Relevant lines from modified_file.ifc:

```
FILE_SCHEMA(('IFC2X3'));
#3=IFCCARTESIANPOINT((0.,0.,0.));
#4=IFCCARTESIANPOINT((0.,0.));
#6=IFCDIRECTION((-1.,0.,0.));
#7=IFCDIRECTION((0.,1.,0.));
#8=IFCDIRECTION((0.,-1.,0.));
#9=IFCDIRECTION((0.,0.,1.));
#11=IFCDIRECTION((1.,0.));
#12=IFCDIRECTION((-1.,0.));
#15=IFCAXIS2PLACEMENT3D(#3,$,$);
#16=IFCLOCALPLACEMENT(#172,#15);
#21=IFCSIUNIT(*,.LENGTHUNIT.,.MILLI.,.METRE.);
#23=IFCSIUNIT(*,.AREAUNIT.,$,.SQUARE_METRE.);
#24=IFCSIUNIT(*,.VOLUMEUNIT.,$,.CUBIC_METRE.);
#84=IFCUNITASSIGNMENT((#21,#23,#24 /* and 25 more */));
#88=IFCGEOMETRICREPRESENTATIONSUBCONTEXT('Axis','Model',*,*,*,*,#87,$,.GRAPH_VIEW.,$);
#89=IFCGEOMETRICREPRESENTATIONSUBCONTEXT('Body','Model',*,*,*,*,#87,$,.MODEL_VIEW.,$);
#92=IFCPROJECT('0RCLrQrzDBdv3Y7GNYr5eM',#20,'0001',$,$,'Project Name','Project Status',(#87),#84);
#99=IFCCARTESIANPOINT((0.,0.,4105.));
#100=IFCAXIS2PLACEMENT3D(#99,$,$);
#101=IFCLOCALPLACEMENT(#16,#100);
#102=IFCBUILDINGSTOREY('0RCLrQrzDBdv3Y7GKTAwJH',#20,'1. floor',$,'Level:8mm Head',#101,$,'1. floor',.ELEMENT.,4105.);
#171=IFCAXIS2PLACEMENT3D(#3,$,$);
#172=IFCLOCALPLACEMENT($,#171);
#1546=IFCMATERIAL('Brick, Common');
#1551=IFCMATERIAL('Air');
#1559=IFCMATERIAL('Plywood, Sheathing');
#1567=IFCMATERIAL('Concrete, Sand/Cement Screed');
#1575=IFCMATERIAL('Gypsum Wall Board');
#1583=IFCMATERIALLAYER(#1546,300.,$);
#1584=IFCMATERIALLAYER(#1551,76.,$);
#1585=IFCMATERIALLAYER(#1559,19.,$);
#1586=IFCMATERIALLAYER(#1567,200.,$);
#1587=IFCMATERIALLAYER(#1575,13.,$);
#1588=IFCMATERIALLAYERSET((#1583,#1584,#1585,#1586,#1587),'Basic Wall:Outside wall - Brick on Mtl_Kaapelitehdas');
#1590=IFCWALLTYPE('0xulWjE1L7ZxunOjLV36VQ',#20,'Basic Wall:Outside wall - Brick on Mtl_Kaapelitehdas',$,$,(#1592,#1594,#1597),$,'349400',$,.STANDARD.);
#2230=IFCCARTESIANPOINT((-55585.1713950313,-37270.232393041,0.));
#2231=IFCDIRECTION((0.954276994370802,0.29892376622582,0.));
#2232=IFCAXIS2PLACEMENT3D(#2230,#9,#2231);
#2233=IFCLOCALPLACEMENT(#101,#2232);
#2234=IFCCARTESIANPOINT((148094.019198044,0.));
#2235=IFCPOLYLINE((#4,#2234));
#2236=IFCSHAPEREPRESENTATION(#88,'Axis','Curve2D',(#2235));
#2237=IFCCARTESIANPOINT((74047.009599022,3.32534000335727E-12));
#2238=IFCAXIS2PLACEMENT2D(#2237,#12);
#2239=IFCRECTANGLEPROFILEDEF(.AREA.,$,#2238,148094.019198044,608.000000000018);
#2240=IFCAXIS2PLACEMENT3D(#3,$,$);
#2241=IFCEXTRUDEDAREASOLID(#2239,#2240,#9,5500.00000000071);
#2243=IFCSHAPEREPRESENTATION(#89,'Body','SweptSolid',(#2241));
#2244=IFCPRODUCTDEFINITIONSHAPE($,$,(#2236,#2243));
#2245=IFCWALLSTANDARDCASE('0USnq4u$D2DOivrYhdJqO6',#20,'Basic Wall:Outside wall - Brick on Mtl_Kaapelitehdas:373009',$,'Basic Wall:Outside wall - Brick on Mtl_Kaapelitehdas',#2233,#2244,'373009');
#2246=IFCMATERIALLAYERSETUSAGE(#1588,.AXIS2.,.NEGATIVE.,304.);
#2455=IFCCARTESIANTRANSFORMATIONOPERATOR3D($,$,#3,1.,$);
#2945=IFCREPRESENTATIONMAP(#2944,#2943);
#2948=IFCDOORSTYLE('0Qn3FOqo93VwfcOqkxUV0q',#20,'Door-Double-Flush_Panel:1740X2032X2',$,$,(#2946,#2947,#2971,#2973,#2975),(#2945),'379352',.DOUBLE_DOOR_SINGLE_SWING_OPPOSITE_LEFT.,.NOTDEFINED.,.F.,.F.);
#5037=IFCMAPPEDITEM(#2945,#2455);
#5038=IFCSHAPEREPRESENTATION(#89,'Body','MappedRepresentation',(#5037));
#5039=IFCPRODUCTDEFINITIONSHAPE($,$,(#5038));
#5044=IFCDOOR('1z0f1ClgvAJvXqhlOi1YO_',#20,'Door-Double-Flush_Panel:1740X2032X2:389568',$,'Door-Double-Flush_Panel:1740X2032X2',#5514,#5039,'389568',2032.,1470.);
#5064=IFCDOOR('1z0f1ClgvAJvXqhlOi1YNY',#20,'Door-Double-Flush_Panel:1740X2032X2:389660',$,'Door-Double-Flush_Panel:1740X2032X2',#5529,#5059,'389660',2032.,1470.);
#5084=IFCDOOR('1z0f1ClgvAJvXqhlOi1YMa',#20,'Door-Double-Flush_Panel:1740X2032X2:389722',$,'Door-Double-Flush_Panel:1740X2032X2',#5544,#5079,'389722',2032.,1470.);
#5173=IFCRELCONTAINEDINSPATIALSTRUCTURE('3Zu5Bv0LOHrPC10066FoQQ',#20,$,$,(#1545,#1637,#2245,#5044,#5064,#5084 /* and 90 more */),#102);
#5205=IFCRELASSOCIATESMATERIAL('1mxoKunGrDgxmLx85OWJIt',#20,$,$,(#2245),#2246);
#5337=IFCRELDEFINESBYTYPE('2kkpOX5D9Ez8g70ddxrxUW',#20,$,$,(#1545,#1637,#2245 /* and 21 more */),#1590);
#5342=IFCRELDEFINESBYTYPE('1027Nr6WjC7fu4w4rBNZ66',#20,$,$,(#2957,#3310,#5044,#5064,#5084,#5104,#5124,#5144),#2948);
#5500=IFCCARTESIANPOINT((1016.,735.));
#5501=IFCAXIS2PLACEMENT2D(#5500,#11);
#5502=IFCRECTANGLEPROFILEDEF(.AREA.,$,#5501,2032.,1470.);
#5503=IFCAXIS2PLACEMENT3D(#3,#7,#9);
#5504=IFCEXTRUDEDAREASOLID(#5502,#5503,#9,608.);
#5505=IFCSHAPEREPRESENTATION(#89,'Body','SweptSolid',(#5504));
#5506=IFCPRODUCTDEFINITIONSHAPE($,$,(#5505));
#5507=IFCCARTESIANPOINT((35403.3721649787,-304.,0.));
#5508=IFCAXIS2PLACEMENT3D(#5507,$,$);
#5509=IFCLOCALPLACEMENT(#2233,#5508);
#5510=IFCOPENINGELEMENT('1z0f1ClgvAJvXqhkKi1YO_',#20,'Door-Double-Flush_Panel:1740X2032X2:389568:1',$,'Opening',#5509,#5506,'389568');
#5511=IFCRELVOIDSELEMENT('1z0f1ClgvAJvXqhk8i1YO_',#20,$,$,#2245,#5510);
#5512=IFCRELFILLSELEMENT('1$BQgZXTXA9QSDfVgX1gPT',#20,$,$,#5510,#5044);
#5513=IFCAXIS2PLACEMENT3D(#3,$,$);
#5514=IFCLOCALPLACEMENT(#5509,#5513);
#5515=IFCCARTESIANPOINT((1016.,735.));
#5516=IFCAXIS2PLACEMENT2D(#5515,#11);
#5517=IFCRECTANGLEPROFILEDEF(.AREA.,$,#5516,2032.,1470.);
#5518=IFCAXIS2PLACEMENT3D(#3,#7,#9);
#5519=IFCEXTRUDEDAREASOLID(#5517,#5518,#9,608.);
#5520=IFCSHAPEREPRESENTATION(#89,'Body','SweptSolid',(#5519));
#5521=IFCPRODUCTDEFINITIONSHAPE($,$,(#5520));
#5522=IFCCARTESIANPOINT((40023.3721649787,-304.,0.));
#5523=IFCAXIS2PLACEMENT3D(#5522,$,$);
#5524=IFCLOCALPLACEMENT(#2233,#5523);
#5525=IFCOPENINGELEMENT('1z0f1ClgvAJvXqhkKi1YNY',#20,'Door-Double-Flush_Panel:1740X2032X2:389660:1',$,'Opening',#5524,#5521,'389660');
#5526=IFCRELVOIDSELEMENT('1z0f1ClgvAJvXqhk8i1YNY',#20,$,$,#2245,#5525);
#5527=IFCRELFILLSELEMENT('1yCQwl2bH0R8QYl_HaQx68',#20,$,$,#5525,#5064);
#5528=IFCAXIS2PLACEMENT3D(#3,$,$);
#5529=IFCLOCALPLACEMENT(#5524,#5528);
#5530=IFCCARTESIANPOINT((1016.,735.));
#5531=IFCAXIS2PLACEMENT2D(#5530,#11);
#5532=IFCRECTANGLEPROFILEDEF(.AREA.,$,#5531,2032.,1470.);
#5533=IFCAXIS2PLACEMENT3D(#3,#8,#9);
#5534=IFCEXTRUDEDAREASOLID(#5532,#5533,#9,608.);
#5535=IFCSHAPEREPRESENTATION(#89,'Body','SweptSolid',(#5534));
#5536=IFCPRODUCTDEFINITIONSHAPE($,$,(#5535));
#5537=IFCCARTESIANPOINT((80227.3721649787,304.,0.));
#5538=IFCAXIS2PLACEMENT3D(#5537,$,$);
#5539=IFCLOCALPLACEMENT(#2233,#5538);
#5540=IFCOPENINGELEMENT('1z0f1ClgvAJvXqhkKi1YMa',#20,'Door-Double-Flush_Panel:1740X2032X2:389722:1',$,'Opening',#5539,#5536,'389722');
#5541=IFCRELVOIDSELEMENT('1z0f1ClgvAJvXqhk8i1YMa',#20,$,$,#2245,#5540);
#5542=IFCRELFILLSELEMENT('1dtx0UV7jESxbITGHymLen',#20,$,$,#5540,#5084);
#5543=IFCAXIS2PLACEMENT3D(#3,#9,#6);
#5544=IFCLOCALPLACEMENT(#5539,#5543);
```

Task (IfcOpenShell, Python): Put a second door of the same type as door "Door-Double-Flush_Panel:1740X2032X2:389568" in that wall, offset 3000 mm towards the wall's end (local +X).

```python
import ifcopenshell
import ifcopenshell.api.feature
import ifcopenshell.api.geometry
import ifcopenshell.api.root
import ifcopenshell.geom
import ifcopenshell.util.element
import ifcopenshell.util.placement
import ifcopenshell.util.shape

model = ifcopenshell.open("modified_file.ifc")
settings = ifcopenshell.geom.settings()


def volume(element):
    """Net volume in cubic metres, openings subtracted."""
    shape = ifcopenshell.geom.create_shape(settings, element)
    return ifcopenshell.util.shape.get_volume(shape.geometry)


def reuse_history(source, copy):
    """copy_class also copies each property set's owner history, people and application; keep the originals."""
    for rel in copy.IsDefinedBy:
        if rel.is_a("IfcRelDefinesByProperties") and (history := rel.RelatingPropertyDefinition.OwnerHistory):
            rel.RelatingPropertyDefinition.OwnerHistory = source.OwnerHistory
            ifcopenshell.util.element.remove_deep2(model, history)


door = model.by_guid("1z0f1ClgvAJvXqhlOi1YO_")
opening = door.FillsVoids[0].RelatingOpeningElement
wall = opening.VoidsElements[0].RelatingBuildingElement
before = volume(wall)
shift = ifcopenshell.util.placement.get_local_placement(wall.ObjectPlacement)[:3, 0] * 3000.0

# copy_class copies the void relationship, type, container and properties, but no geometry.
new_opening = ifcopenshell.api.root.copy_class(model, product=opening)
new_opening.Representation = ifcopenshell.util.element.copy_deep(
    model, opening.Representation, exclude=["IfcGeometricRepresentationContext", "IfcRepresentationMap"]
)
new_opening.Name = "Door-Double-Flush_Panel:1740X2032X2"
new_opening.Tag = None
new_door = ifcopenshell.api.root.copy_class(model, product=door)
new_door.Representation = ifcopenshell.util.element.copy_deep(
    model, door.Representation, exclude=["IfcGeometricRepresentationContext", "IfcRepresentationMap"]
)
new_door.Name = "Door-Double-Flush_Panel:1740X2032X2"
new_door.Tag = None
reuse_history(door, new_door)
fills = ifcopenshell.api.feature.add_filling(model, opening=new_opening, element=new_door)
fills.OwnerHistory = new_door.OwnerHistory  # required in IFC2X3

for old, new in ((opening, new_opening), (door, new_door)):
    matrix = ifcopenshell.util.placement.get_local_placement(old.ObjectPlacement)
    matrix[:3, 3] += shift
    ifcopenshell.api.geometry.edit_object_placement(model, product=new, matrix=matrix, is_si=False)

after = volume(wall)

print(f"wall volume {before:.3f} -> {after:.3f} m3")

model.write("modified_file_v2.ifc")
```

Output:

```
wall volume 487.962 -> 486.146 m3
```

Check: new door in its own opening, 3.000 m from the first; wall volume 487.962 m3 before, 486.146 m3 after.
